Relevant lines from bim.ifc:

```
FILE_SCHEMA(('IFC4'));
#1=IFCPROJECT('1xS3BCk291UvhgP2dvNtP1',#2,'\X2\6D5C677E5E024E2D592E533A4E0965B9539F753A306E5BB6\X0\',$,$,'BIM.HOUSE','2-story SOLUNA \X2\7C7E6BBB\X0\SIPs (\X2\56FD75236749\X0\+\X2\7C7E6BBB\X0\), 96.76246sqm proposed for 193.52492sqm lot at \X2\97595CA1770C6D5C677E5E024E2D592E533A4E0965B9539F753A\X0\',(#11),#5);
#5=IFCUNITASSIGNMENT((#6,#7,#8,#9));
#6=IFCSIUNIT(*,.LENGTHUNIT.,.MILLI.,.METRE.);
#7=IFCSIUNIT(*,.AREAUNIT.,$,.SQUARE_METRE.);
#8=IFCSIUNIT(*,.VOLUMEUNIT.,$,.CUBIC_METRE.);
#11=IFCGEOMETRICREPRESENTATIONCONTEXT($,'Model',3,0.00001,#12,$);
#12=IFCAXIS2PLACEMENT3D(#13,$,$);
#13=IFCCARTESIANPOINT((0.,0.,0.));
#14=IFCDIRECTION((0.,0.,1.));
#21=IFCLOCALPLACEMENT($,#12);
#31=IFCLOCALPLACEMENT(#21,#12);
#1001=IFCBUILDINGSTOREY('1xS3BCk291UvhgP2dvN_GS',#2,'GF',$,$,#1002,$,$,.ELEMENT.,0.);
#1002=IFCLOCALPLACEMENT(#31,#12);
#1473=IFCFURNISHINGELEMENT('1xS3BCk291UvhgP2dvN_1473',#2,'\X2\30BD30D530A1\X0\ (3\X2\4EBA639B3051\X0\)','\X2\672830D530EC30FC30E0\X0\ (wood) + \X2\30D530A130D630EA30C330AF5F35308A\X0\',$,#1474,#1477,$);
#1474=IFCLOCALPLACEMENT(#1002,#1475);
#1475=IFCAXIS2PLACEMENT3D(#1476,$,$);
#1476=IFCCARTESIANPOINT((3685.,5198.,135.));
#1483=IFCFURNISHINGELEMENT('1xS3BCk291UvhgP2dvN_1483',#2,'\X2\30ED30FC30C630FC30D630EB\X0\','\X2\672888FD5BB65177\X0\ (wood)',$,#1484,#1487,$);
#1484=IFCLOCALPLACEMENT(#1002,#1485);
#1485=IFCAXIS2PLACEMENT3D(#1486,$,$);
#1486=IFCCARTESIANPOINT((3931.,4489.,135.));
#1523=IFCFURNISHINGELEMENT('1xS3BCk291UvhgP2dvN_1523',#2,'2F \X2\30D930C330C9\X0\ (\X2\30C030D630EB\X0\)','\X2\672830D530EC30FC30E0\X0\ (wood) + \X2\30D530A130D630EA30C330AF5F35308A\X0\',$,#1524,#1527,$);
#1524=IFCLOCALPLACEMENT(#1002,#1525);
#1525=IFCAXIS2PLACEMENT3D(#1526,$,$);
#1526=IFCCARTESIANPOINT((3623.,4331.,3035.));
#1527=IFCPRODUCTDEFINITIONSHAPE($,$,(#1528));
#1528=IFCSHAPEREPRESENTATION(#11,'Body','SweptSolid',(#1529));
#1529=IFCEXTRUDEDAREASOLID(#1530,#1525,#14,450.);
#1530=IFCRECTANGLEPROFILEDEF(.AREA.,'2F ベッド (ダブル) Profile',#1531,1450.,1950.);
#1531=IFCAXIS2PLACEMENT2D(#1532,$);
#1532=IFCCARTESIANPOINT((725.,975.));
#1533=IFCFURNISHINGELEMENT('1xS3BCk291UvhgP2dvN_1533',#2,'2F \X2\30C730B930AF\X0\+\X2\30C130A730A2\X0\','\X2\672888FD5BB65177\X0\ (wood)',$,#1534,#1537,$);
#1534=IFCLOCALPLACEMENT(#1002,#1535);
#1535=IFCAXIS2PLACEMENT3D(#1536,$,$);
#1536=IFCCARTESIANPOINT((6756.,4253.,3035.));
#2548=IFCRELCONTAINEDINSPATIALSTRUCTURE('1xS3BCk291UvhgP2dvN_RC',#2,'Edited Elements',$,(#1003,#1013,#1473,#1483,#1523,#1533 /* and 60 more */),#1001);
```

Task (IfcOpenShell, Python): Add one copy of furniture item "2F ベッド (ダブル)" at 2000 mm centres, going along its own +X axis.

```python
import ifcopenshell
import ifcopenshell.api.geometry
import ifcopenshell.api.root
import ifcopenshell.util.element
import ifcopenshell.util.placement
import ifcopenshell.util.unit

model = ifcopenshell.open("bim.ifc")
unit_scale = ifcopenshell.util.unit.calculate_unit_scale(model)


def reuse_history(source, copy):
    """copy_class also copies each property set's owner history, people and application; keep the originals."""
    for rel in copy.IsDefinedBy:
        if rel.is_a("IfcRelDefinesByProperties") and (history := rel.RelatingPropertyDefinition.OwnerHistory):
            rel.RelatingPropertyDefinition.OwnerHistory = source.OwnerHistory
            ifcopenshell.util.element.remove_deep2(model, history)


source = model.by_id(1523)
base = ifcopenshell.util.placement.get_local_placement(source.ObjectPlacement)
step = base[:3, 0] * 2 / unit_scale

for i in range(1, 2):
    copy = ifcopenshell.api.root.copy_class(model, product=source)
    copy.Representation = ifcopenshell.util.element.copy_deep(
        model, source.Representation, exclude=["IfcGeometricRepresentationContext", "IfcRepresentationMap"]
    )
    reuse_history(source, copy)
    matrix = base.copy()
    matrix[:3, 3] += i * step
    print("added at", matrix[:3, 3].round(3) + 0.0)
    ifcopenshell.api.geometry.edit_object_placement(model, product=copy, matrix=matrix, is_si=False)

model.write("bim_rev.ifc")
```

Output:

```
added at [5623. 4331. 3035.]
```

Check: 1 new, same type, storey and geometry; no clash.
